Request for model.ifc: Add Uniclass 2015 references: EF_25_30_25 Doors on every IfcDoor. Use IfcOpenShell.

First a look at what the model holds.

```python
import ifcopenshell

model = ifcopenshell.open("model.ifc")
print(model.schema)
print("classifications:", [c.Name for c in model.by_type("IfcClassification")])
for ifc_class in ("IfcDoor", "IfcRoof", "IfcStair", "IfcWall", "IfcWindow"):
    print(ifc_class, len(model.by_type(ifc_class)))
```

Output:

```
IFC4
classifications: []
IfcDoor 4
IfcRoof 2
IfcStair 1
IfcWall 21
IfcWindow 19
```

```python
import ifcopenshell
import ifcopenshell.api.classification

model = ifcopenshell.open("model.ifc")

system = ifcopenshell.api.classification.add_classification(model, classification="Uniclass 2015")

codes = {
    "IfcDoor": ("EF_25_30_25", "Doors"),
}
for ifc_class, (code, name) in codes.items():
    products = model.by_type(ifc_class)
    ifcopenshell.api.classification.add_reference(
        model, products=products, classification=system, identification=code, name=name
    )
    print(code, len(products))

model.write("model_edited.ifc")
```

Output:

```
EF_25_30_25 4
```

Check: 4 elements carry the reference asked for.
